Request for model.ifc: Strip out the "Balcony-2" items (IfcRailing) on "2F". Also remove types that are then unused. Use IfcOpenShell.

First a look at what the model holds.

```python
import ifcopenshell
import ifcopenshell.util.element

model = ifcopenshell.open("model.ifc")
print(model.schema)
storey = next(s for s in model.by_type("IfcBuildingStorey") if s.Name == "2F")
railings = [e for e in ifcopenshell.util.element.get_decomposition(storey) if e.is_a("IfcRailing")]
seen = {}
for e in railings:
    element_type = ifcopenshell.util.element.get_type(e)
    name = element_type.Name if element_type not in (None, e) else None
    seen[name] = seen.get(name, 0) + 1
for name, count in sorted(seen.items(), key=str):
    print(count, "x", name)
```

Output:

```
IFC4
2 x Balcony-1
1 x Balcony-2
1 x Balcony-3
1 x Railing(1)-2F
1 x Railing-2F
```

```python
import ifcopenshell
import ifcopenshell.api.root
import ifcopenshell.util.element

model = ifcopenshell.open("model.ifc")

storey = next(s for s in model.by_type("IfcBuildingStorey") if s.Name == "2F")
railings = [e for e in ifcopenshell.util.element.get_decomposition(storey) if e.is_a("IfcRailing")]
targets = [e for e in railings if (t := ifcopenshell.util.element.get_type(e)) not in (None, e) and t.Name == "Balcony-2"]
types = {ifcopenshell.util.element.get_type(e) for e in targets} - {None, *targets}

for e in targets:
    ifcopenshell.api.root.remove_product(model, product=e)
print(len(targets), "removed")

unused = [t for t in types if not ifcopenshell.util.element.get_types(t)]
for t in unused:
    ifcopenshell.api.root.remove_product(model, product=t)
print(len(unused), "unused types removed")

model.write("model_edited.ifc")
```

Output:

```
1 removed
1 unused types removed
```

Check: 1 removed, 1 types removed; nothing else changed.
